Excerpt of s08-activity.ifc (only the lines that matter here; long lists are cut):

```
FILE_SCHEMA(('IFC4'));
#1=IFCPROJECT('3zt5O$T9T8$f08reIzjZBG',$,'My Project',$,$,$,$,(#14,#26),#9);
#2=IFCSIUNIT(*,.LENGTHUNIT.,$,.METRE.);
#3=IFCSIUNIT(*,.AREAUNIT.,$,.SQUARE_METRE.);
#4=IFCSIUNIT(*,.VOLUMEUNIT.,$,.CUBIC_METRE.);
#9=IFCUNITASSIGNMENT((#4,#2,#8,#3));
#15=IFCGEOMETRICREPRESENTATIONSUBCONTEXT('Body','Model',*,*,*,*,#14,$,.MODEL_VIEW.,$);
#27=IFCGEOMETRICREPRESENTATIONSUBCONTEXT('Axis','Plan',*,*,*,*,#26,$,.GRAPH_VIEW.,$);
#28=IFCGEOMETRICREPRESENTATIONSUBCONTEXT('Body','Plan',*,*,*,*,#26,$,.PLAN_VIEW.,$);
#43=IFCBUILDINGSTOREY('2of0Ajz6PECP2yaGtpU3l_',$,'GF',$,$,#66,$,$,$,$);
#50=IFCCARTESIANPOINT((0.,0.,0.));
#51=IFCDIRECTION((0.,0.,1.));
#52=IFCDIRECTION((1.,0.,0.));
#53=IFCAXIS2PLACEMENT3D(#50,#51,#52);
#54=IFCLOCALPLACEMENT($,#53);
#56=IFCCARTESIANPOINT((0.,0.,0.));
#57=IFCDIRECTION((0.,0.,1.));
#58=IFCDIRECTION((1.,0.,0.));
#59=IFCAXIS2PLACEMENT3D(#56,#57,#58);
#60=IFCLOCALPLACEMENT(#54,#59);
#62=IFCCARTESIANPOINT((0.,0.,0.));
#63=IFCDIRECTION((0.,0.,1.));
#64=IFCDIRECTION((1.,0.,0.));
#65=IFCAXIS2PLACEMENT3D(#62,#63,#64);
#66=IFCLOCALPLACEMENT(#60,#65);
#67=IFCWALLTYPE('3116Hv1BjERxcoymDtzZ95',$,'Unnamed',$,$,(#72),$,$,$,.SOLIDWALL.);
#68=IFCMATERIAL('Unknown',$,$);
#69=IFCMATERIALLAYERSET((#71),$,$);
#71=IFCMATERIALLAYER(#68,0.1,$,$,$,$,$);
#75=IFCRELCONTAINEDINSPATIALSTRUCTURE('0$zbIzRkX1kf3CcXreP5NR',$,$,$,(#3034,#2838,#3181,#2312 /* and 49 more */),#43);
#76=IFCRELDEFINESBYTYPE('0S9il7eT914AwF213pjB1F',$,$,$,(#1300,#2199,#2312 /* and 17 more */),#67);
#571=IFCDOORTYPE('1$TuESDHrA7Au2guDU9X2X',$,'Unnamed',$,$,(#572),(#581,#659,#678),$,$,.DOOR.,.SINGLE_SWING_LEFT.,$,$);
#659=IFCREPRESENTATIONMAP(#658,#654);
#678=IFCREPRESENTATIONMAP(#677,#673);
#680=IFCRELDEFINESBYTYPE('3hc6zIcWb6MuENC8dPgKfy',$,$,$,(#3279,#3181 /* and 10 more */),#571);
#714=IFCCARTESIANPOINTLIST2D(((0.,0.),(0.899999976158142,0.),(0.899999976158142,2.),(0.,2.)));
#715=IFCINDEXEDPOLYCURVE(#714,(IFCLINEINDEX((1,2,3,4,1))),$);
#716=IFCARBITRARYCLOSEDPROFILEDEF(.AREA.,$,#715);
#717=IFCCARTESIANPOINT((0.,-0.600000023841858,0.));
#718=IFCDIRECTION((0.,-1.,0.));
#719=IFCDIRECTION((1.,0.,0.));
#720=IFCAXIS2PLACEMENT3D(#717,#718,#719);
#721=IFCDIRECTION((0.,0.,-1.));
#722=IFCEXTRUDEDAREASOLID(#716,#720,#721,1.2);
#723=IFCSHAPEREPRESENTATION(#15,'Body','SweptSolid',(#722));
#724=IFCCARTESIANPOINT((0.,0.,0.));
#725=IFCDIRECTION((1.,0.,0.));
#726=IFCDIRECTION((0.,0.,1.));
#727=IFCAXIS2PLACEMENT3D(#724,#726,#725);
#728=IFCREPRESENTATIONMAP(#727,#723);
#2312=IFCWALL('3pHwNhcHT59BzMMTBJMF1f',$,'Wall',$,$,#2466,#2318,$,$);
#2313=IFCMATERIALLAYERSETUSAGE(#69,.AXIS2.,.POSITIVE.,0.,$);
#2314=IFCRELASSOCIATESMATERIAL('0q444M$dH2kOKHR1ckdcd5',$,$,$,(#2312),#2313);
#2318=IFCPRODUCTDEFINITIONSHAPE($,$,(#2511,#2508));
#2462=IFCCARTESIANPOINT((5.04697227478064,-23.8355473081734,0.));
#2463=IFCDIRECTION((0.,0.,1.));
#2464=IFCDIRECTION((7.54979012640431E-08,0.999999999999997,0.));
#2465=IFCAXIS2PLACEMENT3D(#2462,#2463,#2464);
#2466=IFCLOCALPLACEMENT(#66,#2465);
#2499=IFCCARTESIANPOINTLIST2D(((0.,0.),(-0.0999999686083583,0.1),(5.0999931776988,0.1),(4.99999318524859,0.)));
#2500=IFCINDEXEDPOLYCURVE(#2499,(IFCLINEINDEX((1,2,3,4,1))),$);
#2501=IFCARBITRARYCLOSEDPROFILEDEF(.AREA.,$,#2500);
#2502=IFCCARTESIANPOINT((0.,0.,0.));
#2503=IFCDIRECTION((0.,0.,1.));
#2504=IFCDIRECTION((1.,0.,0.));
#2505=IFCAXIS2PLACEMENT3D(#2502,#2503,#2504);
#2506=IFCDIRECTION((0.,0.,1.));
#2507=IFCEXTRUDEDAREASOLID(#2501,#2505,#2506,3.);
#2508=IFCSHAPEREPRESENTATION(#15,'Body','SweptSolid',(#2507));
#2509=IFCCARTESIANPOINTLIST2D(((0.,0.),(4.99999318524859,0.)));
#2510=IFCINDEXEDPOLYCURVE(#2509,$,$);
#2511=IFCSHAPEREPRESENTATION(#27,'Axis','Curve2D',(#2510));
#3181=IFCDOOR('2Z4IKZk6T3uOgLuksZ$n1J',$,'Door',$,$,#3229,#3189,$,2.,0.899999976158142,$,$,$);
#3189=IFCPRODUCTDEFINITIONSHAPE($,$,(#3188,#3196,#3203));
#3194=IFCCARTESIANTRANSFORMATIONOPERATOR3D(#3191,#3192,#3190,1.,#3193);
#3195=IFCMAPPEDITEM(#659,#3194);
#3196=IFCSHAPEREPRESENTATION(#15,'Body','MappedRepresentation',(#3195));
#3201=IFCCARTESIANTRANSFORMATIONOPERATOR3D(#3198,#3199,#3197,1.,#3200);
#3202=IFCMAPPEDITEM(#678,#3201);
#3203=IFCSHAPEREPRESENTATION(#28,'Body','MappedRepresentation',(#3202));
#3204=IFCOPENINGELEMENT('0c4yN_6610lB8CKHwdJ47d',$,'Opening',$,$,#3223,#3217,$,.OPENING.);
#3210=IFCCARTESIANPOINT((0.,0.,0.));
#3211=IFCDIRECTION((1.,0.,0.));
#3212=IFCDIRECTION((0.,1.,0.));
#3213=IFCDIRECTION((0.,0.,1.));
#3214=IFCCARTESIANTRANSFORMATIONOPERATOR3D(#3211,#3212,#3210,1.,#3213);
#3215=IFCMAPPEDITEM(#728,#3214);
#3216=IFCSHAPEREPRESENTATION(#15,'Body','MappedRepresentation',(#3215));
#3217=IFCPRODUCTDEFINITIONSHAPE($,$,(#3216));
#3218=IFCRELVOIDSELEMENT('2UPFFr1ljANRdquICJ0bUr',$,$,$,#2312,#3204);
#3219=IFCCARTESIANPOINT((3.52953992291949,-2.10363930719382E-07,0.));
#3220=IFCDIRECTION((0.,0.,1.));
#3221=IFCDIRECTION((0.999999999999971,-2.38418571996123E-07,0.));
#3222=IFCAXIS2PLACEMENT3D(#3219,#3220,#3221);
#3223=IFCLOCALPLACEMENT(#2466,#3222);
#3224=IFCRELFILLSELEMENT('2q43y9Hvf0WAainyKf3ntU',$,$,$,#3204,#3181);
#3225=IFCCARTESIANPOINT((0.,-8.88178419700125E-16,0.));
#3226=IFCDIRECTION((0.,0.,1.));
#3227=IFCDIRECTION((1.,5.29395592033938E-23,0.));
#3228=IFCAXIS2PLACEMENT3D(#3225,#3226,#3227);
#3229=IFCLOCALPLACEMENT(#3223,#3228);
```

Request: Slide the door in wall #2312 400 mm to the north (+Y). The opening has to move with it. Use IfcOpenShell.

```python
import ifcopenshell
import ifcopenshell.api.geometry
import ifcopenshell.util.placement
import ifcopenshell.util.unit

model = ifcopenshell.open("s08-activity.ifc")
unit_scale = ifcopenshell.util.unit.calculate_unit_scale(model)

door = model.by_guid("2Z4IKZk6T3uOgLuksZ$n1J")
opening = door.FillsVoids[0].RelatingOpeningElement
wall = opening.VoidsElements[0].RelatingBuildingElement

wall_matrix = ifcopenshell.util.placement.get_local_placement(wall.ObjectPlacement)
shift = wall_matrix[:3, 0] * 0.4 / unit_scale
before = ifcopenshell.util.placement.get_local_placement(door.ObjectPlacement)[:3, 3].copy()

# The door is placed relative to its opening, so it follows when the opening moves.
matrix = ifcopenshell.util.placement.get_local_placement(opening.ObjectPlacement)
matrix[:3, 3] += shift
ifcopenshell.api.geometry.edit_object_placement(
    model, product=opening, matrix=matrix, is_si=False, should_transform_children=True
)

after = ifcopenshell.util.placement.get_local_placement(door.ObjectPlacement)[:3, 3]
print("door moved by", (after - before).round(3) + 0.0)

model.write("s08-activity_edited.ifc")
```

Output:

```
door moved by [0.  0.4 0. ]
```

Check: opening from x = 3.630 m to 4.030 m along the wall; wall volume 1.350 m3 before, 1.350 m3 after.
